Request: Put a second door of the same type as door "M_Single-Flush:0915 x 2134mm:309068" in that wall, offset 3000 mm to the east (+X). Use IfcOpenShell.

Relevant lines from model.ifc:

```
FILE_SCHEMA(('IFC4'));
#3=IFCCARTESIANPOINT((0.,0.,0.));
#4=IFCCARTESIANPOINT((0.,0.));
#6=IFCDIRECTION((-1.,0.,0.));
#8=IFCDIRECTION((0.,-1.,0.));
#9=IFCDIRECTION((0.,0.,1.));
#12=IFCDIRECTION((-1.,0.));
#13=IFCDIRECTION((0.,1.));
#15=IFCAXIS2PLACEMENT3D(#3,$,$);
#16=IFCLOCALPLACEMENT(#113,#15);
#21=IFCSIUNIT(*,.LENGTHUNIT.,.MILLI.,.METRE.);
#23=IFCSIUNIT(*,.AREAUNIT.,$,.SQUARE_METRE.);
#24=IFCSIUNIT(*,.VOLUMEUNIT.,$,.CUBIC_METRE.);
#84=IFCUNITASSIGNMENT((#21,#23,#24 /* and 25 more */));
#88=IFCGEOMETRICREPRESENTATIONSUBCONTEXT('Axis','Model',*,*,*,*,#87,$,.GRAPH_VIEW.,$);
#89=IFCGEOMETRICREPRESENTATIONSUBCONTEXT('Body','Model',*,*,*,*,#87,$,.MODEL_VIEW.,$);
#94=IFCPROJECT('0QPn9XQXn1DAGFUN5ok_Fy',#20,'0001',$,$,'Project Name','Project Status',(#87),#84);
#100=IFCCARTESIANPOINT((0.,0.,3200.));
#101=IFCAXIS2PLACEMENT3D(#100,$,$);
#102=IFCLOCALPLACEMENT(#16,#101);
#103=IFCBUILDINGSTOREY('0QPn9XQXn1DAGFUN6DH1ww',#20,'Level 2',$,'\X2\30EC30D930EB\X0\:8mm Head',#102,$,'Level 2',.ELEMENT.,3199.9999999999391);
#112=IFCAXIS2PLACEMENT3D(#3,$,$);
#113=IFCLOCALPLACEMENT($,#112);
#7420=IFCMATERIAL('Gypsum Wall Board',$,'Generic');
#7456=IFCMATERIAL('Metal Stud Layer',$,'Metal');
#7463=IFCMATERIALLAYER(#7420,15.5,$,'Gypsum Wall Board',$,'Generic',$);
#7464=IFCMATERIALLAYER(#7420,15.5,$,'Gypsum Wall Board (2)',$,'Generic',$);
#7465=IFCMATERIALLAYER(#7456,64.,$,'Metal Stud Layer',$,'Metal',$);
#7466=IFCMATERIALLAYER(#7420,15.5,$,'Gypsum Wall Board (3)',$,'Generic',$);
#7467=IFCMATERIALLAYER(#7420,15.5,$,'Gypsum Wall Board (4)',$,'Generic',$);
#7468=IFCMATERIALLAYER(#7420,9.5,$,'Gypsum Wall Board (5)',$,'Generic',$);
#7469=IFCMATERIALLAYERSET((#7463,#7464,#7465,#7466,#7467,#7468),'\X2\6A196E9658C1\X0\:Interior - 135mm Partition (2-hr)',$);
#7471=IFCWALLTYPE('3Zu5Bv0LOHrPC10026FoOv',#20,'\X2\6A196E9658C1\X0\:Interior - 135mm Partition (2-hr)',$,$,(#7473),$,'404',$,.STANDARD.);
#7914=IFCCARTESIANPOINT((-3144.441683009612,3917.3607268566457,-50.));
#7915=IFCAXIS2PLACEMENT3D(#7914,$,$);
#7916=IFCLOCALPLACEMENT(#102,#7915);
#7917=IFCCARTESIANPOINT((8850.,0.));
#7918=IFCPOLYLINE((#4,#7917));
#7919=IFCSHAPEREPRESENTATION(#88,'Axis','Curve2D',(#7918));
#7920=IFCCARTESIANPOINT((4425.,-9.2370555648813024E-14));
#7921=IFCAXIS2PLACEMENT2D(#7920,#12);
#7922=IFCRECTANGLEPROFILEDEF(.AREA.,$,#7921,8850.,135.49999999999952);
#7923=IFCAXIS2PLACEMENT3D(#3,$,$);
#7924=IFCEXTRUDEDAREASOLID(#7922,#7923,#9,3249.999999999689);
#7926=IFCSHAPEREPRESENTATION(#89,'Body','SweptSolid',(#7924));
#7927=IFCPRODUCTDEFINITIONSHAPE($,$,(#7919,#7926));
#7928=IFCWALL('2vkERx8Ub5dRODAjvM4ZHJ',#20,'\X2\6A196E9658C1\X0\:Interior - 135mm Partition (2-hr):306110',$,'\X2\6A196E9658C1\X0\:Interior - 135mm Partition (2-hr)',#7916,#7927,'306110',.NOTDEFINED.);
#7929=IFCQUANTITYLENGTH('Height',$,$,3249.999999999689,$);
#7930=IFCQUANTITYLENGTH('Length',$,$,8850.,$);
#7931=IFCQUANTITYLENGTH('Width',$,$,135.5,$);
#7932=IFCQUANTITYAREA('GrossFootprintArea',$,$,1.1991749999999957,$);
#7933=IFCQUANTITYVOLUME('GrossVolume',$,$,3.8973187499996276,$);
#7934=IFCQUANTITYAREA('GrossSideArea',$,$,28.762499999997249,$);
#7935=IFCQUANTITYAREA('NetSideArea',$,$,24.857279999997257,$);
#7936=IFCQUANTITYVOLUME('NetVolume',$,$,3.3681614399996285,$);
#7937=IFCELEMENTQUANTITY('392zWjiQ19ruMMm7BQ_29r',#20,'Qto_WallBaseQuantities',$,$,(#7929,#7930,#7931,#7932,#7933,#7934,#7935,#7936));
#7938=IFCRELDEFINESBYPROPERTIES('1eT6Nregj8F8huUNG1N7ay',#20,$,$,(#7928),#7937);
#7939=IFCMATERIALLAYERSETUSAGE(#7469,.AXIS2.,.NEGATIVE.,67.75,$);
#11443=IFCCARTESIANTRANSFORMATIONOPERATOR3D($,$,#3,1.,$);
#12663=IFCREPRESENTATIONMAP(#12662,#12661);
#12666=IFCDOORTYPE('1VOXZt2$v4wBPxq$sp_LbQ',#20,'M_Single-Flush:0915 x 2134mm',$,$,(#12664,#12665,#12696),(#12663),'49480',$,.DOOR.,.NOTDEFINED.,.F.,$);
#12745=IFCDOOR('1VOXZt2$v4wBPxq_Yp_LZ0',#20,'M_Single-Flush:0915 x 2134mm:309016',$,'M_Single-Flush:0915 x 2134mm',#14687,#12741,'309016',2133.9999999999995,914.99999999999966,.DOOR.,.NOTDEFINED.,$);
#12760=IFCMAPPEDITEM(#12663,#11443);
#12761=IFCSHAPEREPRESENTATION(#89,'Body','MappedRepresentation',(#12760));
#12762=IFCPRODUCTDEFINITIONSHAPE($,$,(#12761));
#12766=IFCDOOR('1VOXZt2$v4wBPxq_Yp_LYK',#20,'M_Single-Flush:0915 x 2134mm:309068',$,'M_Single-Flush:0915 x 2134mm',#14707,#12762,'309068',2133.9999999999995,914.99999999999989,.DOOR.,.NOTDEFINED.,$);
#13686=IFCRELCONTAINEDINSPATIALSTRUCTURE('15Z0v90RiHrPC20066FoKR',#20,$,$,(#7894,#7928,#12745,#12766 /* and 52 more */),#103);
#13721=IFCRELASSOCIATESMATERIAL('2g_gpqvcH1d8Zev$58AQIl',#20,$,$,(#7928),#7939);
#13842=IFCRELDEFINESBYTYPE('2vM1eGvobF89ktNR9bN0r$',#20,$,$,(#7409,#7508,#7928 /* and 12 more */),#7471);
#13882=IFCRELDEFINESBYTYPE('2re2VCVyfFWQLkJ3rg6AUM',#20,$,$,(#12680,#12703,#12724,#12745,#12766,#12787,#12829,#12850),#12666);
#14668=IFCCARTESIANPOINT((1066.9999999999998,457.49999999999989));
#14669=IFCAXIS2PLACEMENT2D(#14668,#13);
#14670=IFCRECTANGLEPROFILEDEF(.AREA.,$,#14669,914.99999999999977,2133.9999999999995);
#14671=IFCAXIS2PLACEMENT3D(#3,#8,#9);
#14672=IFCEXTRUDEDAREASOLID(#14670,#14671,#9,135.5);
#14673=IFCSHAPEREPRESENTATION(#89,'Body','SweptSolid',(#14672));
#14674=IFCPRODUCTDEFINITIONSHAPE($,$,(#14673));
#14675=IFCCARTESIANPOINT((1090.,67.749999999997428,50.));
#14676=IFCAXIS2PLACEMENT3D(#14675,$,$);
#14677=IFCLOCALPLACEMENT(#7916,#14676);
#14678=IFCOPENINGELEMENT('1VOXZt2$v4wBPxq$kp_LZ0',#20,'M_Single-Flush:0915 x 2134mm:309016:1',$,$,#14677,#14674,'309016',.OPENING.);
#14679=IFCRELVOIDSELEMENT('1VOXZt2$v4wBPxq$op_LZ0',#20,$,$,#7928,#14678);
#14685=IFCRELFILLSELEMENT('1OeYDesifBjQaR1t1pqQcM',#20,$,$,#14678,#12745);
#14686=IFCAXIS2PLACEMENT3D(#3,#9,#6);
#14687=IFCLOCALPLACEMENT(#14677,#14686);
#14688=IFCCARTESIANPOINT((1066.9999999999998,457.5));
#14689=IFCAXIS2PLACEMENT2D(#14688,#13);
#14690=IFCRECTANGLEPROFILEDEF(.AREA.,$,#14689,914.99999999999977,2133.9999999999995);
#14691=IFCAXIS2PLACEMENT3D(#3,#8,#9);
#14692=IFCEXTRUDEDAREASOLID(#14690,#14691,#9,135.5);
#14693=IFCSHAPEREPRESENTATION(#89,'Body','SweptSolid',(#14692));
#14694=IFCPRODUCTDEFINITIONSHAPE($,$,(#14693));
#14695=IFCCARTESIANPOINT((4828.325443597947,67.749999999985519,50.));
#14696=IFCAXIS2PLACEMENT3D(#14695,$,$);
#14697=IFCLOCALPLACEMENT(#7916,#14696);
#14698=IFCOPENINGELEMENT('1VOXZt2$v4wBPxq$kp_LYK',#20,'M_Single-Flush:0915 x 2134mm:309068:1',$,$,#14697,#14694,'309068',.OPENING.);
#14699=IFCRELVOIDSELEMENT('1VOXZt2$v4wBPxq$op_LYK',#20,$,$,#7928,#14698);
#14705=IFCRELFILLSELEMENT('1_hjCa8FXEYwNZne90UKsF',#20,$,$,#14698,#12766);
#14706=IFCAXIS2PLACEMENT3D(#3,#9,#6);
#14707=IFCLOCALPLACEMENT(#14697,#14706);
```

```python
import ifcopenshell
import ifcopenshell.api.feature
import ifcopenshell.api.geometry
import ifcopenshell.api.pset
import ifcopenshell.api.root
import ifcopenshell.geom
import ifcopenshell.util.element
import ifcopenshell.util.placement
import ifcopenshell.util.shape
import ifcopenshell.util.unit

model = ifcopenshell.open("model.ifc")
area_scale = ifcopenshell.util.unit.calculate_unit_scale(model, "AREAUNIT")
volume_scale = ifcopenshell.util.unit.calculate_unit_scale(model, "VOLUMEUNIT")
settings = ifcopenshell.geom.settings()


def volume(element):
    """Net volume in cubic metres, openings subtracted."""
    shape = ifcopenshell.geom.create_shape(settings, element)
    return ifcopenshell.util.shape.get_volume(shape.geometry)


def reuse_history(source, copy):
    """copy_class also copies each property set's owner history, people and application; keep the originals."""
    for rel in copy.IsDefinedBy:
        if rel.is_a("IfcRelDefinesByProperties") and (history := rel.RelatingPropertyDefinition.OwnerHistory):
            rel.RelatingPropertyDefinition.OwnerHistory = source.OwnerHistory
            ifcopenshell.util.element.remove_deep2(model, history)


door = model.by_id(12766)
opening = door.FillsVoids[0].RelatingOpeningElement
wall = opening.VoidsElements[0].RelatingBuildingElement
before = volume(wall)
shift = ifcopenshell.util.placement.get_local_placement(wall.ObjectPlacement)[:3, 0] * 3000.0

# copy_class copies the void relationship, type, container and properties, but no geometry.
new_opening = ifcopenshell.api.root.copy_class(model, product=opening)
new_opening.Representation = ifcopenshell.util.element.copy_deep(
    model, opening.Representation, exclude=["IfcGeometricRepresentationContext", "IfcRepresentationMap"]
)
new_opening.Name = "M_Single-Flush:0915 x 2134mm"
new_opening.Tag = None
reuse_history(opening, new_opening)
new_door = ifcopenshell.api.root.copy_class(model, product=door)
new_door.Representation = ifcopenshell.util.element.copy_deep(
    model, door.Representation, exclude=["IfcGeometricRepresentationContext", "IfcRepresentationMap"]
)
new_door.Name = "M_Single-Flush:0915 x 2134mm"
new_door.Tag = None
reuse_history(door, new_door)
ifcopenshell.api.feature.add_filling(model, opening=new_opening, element=new_door)

for old, new in ((opening, new_opening), (door, new_door)):
    matrix = ifcopenshell.util.placement.get_local_placement(old.ObjectPlacement)
    matrix[:3, 3] += shift
    ifcopenshell.api.geometry.edit_object_placement(model, product=new, matrix=matrix, is_si=False)

after = volume(wall)
thickness = 0.1355  # wall thickness in metres

# Update the wall's stored quantities.
qto = model.by_id(ifcopenshell.util.element.get_pset(wall, "Qto_WallBaseQuantities", should_inherit=False)["id"])
ifcopenshell.api.pset.edit_qto(model, qto=qto, properties={
    "NetSideArea": after / thickness / area_scale,
    "NetVolume": after / volume_scale,
})

print(f"wall volume {before:.3f} -> {after:.3f} m3")

model.write("model_v2.ifc")
```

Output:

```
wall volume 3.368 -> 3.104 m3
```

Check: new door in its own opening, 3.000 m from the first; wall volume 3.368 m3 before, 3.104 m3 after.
